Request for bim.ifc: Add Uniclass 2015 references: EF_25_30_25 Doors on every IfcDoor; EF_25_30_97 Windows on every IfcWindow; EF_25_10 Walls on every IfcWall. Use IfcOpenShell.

First a look at what the model holds.

```python
import ifcopenshell

model = ifcopenshell.open("bim.ifc")
print(model.schema)
print("classifications:", [c.Name for c in model.by_type("IfcClassification")])
for ifc_class in ("IfcDoor", "IfcRoof", "IfcStair", "IfcWall", "IfcWindow"):
    print(ifc_class, len(model.by_type(ifc_class)))
```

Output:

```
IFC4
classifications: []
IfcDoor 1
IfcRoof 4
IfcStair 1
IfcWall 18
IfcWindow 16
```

```python
import ifcopenshell
import ifcopenshell.api.classification

model = ifcopenshell.open("bim.ifc")

system = ifcopenshell.api.classification.add_classification(model, classification="Uniclass 2015")

codes = {
    "IfcDoor": ("EF_25_30_25", "Doors"),
    "IfcWindow": ("EF_25_30_97", "Windows"),
    "IfcWall": ("EF_25_10", "Walls"),
}
for ifc_class, (code, name) in codes.items():
    products = model.by_type(ifc_class)
    ifcopenshell.api.classification.add_reference(
        model, products=products, classification=system, identification=code, name=name
    )
    print(code, len(products))

model.write("bim_edited.ifc")
```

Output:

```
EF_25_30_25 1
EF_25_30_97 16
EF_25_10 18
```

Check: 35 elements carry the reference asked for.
